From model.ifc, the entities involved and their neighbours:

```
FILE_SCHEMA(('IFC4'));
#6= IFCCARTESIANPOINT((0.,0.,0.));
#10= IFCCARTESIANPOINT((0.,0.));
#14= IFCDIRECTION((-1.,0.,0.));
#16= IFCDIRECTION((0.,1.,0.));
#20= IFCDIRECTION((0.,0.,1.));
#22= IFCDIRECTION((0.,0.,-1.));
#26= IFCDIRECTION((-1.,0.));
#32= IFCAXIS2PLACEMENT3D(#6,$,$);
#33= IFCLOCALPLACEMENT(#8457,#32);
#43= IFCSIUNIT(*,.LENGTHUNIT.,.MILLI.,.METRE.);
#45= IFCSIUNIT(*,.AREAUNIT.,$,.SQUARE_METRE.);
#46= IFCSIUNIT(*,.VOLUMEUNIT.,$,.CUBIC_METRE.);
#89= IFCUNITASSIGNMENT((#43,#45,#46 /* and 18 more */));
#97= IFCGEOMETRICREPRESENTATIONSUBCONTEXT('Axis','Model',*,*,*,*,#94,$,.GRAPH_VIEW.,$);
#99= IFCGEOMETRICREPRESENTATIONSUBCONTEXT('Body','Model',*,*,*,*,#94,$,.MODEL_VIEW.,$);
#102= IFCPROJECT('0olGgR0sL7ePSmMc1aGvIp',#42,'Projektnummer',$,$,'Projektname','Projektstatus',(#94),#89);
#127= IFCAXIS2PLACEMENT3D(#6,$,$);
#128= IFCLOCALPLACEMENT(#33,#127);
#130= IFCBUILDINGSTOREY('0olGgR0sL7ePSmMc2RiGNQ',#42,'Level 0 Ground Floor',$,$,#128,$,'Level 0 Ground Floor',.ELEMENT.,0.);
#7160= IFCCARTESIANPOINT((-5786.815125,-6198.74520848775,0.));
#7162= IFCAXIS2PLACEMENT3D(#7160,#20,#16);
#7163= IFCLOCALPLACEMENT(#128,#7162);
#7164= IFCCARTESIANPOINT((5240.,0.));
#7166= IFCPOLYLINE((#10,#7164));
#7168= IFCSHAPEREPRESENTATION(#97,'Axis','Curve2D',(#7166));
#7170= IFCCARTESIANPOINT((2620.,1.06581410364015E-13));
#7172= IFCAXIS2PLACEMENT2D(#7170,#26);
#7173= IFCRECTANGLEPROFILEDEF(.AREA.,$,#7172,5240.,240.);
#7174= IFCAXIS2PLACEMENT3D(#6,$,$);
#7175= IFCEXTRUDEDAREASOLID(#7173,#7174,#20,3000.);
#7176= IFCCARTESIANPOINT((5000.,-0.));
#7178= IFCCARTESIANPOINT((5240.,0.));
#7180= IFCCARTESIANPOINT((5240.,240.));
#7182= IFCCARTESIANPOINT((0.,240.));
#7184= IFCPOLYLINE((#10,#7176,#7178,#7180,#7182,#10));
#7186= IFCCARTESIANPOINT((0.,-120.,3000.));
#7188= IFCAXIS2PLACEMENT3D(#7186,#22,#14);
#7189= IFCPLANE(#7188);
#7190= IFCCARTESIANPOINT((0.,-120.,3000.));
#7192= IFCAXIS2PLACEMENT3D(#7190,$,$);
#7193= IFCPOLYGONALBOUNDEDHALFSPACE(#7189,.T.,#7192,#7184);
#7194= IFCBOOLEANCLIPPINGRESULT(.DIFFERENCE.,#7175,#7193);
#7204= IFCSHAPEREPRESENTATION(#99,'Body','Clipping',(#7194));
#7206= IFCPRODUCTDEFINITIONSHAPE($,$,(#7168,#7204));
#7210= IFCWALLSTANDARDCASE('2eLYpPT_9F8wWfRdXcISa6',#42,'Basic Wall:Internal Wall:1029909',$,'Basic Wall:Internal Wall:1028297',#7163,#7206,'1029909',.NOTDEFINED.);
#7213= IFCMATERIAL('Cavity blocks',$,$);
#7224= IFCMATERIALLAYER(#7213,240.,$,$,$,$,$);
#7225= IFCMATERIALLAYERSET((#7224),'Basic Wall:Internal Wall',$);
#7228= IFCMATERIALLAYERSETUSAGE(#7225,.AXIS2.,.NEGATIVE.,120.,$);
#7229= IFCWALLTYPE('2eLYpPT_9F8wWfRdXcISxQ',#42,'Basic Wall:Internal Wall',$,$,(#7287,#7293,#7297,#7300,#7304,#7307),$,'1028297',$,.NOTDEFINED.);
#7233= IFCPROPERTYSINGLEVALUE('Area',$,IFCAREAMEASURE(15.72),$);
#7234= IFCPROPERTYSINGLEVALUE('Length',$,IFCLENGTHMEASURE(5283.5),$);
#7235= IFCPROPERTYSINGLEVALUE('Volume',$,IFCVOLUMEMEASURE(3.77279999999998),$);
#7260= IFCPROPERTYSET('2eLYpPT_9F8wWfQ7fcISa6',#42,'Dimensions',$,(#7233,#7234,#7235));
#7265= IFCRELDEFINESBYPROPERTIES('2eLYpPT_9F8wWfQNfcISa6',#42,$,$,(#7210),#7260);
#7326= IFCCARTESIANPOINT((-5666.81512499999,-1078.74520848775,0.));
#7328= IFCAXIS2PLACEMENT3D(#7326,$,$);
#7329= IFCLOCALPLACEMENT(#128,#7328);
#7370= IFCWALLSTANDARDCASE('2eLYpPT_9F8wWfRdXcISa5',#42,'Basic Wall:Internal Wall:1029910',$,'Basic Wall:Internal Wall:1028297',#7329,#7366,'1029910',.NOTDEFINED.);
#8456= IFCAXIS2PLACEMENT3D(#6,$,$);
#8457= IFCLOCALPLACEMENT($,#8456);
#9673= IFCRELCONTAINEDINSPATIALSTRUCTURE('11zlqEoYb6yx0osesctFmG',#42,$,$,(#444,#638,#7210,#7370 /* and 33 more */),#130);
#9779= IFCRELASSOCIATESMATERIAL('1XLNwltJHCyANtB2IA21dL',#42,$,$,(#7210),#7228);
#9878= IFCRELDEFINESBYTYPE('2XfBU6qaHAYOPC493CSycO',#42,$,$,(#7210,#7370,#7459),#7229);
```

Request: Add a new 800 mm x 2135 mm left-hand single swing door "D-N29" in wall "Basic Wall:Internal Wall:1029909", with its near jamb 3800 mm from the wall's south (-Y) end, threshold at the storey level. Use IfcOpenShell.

```python
import numpy as np
import ifcopenshell
import ifcopenshell.api.feature
import ifcopenshell.api.geometry
import ifcopenshell.api.pset
import ifcopenshell.api.root
import ifcopenshell.api.spatial
import ifcopenshell.geom
import ifcopenshell.util.element
import ifcopenshell.util.placement
import ifcopenshell.util.representation
import ifcopenshell.util.shape
import ifcopenshell.util.unit

model = ifcopenshell.open("model.ifc")
unit_scale = ifcopenshell.util.unit.calculate_unit_scale(model)
area_scale = ifcopenshell.util.unit.calculate_unit_scale(model, "AREAUNIT")
volume_scale = ifcopenshell.util.unit.calculate_unit_scale(model, "VOLUMEUNIT")
settings = ifcopenshell.geom.settings()


def volume(element):
    """Net volume in cubic metres, openings subtracted."""
    shape = ifcopenshell.geom.create_shape(settings, element)
    return ifcopenshell.util.shape.get_volume(shape.geometry)


wall = model.by_guid("2eLYpPT_9F8wWfRdXcISa6")
storey = ifcopenshell.util.element.get_container(wall, ifc_class="IfcBuildingStorey")
context = ifcopenshell.util.representation.get_context(model, "Model", "Body", "MODEL_VIEW")
before = volume(wall)

width, height, from_end, sill = 0.8, 2.135, 3.8, 0.0  # metres

# The wall runs along its own X axis, and the end named is its -X end.
wall_shape = ifcopenshell.geom.create_shape(settings, wall)
x, y, z = ifcopenshell.util.shape.get_vertices(wall_shape.geometry).T
start = x.min() + from_end
face, thickness = float(y.min()), float(y.max() - y.min())
wall_matrix = ifcopenshell.util.placement.get_local_placement(wall.ObjectPlacement)
level = ifcopenshell.util.placement.get_local_placement(storey.ObjectPlacement)[2, 3]


def in_wall(x, y):
    """Placement at x, y metres in the wall's axes, at sill height."""
    matrix = wall_matrix.copy()
    matrix[:, 3] = wall_matrix @ np.array([x / unit_scale, y / unit_scale, 0.0, 1.0])
    matrix[2, 3] = level + sill / unit_scale
    return matrix


# Opening: a box that overshoots both wall faces by 50 mm.
opening = ifcopenshell.api.root.create_entity(model, ifc_class="IfcOpeningElement", predefined_type="OPENING")
box = ifcopenshell.api.geometry.add_wall_representation(
    model, context=context, length=width, height=height, thickness=thickness + 0.1
)
ifcopenshell.api.geometry.assign_representation(model, product=opening, representation=box)
ifcopenshell.api.geometry.edit_object_placement(model, product=opening, matrix=in_wall(start, face - 0.05), is_si=False)
ifcopenshell.api.feature.add_feature(model, feature=opening, element=wall)

door = ifcopenshell.api.root.create_entity(model, ifc_class="IfcDoor", name="D-N29", predefined_type="DOOR")
door.OverallWidth, door.OverallHeight = width / unit_scale, height / unit_scale
door.OperationType = "SINGLE_SWING_LEFT"
body = ifcopenshell.api.geometry.add_door_representation(
    model,
    context=context,
    overall_width=door.OverallWidth,
    overall_height=door.OverallHeight,
    operation_type="SINGLE_SWING_LEFT",
    lining_properties={"LiningDepth": thickness / unit_scale, "ThresholdDepth": thickness / unit_scale},
)
ifcopenshell.api.geometry.assign_representation(model, product=door, representation=body)
ifcopenshell.api.spatial.assign_container(model, products=[door], relating_structure=storey)
ifcopenshell.api.feature.add_filling(model, opening=opening, element=door)

# The lining spans the wall, so the door starts at the wall face.
ifcopenshell.api.geometry.edit_object_placement(model, product=door, matrix=in_wall(start, face), is_si=False)

after = volume(wall)

# Update the wall's stored quantities.
pset = model.by_id(ifcopenshell.util.element.get_pset(wall, "Dimensions", should_inherit=False)["id"])
ifcopenshell.api.pset.edit_pset(model, pset=pset, properties={
    "Area": model.create_entity("IfcAreaMeasure", after / thickness / area_scale),
    "Volume": model.create_entity("IfcVolumeMeasure", after / volume_scale),
})

print(f"wall volume {before:.3f} -> {after:.3f} m3")

model.write("model_updated.ifc")
```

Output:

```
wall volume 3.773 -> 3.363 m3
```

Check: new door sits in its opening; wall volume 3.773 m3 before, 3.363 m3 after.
